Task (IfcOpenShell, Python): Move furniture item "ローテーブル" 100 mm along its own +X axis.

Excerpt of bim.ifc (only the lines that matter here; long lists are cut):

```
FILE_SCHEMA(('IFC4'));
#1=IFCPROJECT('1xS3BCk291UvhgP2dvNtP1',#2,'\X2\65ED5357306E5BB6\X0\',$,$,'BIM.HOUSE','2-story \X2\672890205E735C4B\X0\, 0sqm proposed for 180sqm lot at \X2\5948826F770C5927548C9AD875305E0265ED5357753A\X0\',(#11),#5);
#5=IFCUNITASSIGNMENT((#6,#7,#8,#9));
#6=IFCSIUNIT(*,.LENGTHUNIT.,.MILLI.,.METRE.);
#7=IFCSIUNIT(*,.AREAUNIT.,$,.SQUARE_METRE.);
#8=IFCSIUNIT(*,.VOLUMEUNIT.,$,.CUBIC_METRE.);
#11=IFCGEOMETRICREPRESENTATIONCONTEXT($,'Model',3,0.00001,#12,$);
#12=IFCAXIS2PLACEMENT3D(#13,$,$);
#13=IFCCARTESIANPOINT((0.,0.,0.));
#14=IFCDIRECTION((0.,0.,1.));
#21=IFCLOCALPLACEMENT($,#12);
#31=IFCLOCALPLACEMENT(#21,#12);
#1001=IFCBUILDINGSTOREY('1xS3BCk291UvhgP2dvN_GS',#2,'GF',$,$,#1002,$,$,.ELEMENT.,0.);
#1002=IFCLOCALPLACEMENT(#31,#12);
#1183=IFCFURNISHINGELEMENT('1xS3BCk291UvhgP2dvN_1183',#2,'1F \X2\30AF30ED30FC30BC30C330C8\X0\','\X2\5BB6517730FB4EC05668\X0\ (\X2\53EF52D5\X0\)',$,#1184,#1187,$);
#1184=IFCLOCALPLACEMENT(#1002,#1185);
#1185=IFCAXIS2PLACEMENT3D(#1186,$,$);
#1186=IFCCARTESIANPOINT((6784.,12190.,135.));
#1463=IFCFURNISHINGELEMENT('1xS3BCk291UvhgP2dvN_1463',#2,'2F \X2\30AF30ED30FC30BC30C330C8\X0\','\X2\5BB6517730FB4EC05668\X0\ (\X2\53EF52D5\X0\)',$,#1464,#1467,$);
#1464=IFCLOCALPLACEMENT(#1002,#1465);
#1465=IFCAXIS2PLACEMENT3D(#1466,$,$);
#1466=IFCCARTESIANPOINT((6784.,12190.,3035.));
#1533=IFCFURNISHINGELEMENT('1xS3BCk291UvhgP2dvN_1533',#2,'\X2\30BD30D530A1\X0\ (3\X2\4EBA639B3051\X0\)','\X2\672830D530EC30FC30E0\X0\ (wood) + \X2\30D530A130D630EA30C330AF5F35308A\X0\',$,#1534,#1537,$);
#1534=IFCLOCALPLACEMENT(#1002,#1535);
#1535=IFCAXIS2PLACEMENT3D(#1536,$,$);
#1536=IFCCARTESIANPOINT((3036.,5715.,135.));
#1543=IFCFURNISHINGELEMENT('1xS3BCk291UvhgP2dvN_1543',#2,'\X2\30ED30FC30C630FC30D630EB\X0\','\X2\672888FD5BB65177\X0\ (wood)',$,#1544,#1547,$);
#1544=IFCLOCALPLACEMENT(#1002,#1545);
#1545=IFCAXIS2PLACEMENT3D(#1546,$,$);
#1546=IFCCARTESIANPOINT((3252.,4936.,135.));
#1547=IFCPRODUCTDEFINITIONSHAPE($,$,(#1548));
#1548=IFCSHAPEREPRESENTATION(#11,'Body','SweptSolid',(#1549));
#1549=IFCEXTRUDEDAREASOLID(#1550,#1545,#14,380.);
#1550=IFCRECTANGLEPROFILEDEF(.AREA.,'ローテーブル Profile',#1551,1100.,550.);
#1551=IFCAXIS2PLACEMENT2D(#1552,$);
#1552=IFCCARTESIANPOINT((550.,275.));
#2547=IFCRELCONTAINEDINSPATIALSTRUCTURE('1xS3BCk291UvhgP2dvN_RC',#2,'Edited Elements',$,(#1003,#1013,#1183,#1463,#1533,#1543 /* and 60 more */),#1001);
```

```python
import ifcopenshell
import ifcopenshell.api.geometry
import ifcopenshell.util.placement

model = ifcopenshell.open("bim.ifc")

item = model.by_guid("1xS3BCk291UvhgP2dvN_1543")
matrix = ifcopenshell.util.placement.get_local_placement(item.ObjectPlacement)
matrix[:3, 3] += matrix[:3, 0] * 100.0
ifcopenshell.api.geometry.edit_object_placement(model, product=item, matrix=matrix, is_si=False)

print(ifcopenshell.util.placement.get_local_placement(item.ObjectPlacement).round(3) + 0.0)

model.write("bim-out.ifc")
```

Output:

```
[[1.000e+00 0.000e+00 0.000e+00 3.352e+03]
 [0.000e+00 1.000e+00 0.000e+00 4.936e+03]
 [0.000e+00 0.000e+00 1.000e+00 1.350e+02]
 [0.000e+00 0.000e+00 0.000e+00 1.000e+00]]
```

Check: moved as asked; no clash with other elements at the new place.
